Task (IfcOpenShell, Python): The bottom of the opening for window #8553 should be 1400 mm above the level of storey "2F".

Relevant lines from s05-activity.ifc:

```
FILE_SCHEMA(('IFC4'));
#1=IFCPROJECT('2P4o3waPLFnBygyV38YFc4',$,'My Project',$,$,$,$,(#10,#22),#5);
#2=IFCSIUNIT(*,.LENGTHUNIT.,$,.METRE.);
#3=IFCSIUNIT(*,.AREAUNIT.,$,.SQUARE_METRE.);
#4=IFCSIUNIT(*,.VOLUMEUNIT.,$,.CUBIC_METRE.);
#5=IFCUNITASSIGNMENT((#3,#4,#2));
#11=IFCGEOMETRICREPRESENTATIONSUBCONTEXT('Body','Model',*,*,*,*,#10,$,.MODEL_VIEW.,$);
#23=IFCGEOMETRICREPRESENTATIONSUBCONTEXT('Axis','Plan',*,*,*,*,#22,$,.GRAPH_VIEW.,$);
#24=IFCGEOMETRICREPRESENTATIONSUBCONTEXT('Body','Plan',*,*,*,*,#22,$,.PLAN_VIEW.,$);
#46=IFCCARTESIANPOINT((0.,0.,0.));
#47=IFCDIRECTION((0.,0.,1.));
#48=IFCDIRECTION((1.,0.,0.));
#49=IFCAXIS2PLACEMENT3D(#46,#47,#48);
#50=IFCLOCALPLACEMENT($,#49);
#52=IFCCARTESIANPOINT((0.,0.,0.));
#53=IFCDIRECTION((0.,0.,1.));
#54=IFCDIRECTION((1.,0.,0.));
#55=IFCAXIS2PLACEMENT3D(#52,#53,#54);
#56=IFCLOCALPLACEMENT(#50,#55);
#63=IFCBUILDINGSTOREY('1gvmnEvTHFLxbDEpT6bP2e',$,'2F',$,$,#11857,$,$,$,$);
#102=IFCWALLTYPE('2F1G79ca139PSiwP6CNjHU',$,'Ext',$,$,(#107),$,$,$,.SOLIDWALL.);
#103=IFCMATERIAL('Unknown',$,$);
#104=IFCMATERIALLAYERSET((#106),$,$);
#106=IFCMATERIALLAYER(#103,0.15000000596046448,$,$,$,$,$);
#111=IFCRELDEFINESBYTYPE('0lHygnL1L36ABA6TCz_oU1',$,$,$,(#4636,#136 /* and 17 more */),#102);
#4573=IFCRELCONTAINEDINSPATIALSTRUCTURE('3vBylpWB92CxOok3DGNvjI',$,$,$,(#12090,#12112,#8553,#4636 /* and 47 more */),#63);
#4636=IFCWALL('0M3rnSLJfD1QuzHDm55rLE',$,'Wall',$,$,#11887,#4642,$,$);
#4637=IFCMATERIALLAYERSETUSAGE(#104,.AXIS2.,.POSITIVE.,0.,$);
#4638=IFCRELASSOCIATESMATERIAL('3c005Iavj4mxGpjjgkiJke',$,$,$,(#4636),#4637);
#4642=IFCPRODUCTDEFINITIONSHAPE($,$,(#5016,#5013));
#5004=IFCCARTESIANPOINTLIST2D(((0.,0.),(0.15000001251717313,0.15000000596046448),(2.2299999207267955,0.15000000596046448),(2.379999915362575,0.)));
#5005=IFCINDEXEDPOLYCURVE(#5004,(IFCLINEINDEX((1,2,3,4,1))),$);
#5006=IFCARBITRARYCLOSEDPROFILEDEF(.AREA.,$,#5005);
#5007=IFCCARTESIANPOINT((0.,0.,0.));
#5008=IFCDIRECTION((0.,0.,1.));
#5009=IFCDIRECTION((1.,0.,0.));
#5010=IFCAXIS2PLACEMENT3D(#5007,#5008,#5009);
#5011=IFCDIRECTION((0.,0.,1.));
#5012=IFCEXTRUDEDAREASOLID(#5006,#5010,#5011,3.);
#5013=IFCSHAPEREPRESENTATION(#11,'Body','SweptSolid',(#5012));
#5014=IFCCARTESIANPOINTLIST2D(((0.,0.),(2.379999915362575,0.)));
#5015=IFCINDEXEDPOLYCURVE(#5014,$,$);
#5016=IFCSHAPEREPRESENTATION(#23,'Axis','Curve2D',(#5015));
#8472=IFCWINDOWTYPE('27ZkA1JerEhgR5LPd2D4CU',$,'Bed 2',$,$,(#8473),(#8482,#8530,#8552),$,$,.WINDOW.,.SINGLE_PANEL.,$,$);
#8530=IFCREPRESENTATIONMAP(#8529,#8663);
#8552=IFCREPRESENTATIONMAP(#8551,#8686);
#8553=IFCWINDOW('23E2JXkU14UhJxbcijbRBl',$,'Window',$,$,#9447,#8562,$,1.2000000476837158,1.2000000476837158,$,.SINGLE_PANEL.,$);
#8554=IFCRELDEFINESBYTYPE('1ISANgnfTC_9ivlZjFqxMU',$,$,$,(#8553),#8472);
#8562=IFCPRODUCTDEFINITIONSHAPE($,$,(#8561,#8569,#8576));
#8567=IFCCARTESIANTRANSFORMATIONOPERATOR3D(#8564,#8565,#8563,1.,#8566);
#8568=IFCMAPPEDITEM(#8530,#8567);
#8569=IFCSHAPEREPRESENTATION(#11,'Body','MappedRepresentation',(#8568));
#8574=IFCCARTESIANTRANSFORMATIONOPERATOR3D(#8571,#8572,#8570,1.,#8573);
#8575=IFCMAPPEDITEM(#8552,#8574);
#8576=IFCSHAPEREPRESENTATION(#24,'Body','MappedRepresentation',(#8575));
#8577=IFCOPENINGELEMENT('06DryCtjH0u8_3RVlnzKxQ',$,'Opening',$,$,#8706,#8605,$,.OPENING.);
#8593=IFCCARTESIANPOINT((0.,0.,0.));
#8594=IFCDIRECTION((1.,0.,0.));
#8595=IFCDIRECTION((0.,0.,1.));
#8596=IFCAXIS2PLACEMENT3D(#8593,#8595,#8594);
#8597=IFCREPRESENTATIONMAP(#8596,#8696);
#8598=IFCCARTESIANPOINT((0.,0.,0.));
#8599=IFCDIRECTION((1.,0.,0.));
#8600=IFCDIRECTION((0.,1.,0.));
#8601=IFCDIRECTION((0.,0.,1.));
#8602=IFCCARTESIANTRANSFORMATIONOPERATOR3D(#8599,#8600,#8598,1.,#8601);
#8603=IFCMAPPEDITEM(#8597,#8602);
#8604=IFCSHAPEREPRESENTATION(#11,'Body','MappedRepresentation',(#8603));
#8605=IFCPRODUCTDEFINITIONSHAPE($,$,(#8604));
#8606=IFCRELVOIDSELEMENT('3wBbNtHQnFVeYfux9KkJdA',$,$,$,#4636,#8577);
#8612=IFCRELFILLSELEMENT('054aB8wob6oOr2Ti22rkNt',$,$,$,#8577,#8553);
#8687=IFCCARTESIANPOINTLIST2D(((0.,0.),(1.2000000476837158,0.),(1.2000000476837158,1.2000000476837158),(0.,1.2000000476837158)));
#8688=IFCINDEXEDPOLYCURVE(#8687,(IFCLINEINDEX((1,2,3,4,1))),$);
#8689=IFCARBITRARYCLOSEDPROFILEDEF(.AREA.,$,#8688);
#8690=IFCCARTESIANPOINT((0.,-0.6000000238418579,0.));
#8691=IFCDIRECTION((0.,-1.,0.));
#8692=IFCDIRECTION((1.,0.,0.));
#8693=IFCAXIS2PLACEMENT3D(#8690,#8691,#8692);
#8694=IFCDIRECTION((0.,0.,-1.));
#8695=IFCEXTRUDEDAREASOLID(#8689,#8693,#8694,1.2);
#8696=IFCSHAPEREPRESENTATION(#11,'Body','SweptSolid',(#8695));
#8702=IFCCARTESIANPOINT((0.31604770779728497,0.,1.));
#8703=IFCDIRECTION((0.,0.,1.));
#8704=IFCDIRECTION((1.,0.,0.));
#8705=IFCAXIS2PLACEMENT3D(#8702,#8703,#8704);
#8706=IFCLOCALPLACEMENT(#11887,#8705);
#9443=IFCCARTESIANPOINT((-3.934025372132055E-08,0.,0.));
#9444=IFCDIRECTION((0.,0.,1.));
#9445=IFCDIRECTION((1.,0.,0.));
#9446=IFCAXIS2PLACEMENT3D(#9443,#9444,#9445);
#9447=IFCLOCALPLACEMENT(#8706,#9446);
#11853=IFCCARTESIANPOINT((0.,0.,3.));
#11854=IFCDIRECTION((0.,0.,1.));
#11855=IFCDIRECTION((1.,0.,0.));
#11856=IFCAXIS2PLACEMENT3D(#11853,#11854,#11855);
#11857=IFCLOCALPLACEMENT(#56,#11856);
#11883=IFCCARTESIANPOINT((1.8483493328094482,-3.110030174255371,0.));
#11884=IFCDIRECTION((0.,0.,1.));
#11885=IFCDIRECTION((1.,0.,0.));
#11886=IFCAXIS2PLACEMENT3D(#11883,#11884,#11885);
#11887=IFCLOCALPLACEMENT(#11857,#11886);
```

```python
import numpy as np
import ifcopenshell
import ifcopenshell.api.geometry
import ifcopenshell.geom
import ifcopenshell.util.element
import ifcopenshell.util.placement
import ifcopenshell.util.shape
import ifcopenshell.util.unit

model = ifcopenshell.open("s05-activity.ifc")
unit_scale = ifcopenshell.util.unit.calculate_unit_scale(model)

window = model.by_id(8553)
opening = window.FillsVoids[0].RelatingOpeningElement
storey = ifcopenshell.util.element.get_container(window, ifc_class="IfcBuildingStorey")
level = ifcopenshell.util.placement.get_local_placement(storey.ObjectPlacement)[2, 3]

# The opening's origin need not be at the sill, so measure its lowest point.
shape = ifcopenshell.geom.create_shape(ifcopenshell.geom.settings(), opening)
bottom = ifcopenshell.util.shape.get_shape_bottom_elevation(shape, shape.geometry) / unit_scale
dz = level + 1.4 - bottom

shift = np.array([0.0, 0.0, dz])
# The window is placed relative to its opening, so it follows when the opening moves.
matrix = ifcopenshell.util.placement.get_local_placement(opening.ObjectPlacement)
matrix[:3, 3] += shift
ifcopenshell.api.geometry.edit_object_placement(
    model, product=opening, matrix=matrix, is_si=False, should_transform_children=True
)

print(f"moved by {dz * unit_scale:+.3f} m")

model.write("s05-activity_rev.ifc")
```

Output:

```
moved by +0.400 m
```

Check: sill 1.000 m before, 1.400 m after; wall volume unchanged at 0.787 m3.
